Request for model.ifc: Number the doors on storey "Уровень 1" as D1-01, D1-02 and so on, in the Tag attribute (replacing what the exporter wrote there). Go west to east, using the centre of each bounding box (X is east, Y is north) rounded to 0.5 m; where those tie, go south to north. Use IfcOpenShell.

First a look at what the model holds.

```python
import ifcopenshell
import ifcopenshell.util.element
import ifcopenshell.util.placement

model = ifcopenshell.open("model.ifc")
print(model.schema)
storey = next(s for s in model.by_type("IfcBuildingStorey") if s.Name == "Уровень 1")
doors = [e for e in ifcopenshell.util.element.get_decomposition(storey) if e.is_a("IfcDoor")]
for e in sorted(doors, key=lambda e: e.id()):
    origin = ifcopenshell.util.placement.get_local_placement(e.ObjectPlacement)[:3, 3]
    print(e.id(), e.Tag, e.Name, origin.round(2) + 0.0, sep=" | ")
```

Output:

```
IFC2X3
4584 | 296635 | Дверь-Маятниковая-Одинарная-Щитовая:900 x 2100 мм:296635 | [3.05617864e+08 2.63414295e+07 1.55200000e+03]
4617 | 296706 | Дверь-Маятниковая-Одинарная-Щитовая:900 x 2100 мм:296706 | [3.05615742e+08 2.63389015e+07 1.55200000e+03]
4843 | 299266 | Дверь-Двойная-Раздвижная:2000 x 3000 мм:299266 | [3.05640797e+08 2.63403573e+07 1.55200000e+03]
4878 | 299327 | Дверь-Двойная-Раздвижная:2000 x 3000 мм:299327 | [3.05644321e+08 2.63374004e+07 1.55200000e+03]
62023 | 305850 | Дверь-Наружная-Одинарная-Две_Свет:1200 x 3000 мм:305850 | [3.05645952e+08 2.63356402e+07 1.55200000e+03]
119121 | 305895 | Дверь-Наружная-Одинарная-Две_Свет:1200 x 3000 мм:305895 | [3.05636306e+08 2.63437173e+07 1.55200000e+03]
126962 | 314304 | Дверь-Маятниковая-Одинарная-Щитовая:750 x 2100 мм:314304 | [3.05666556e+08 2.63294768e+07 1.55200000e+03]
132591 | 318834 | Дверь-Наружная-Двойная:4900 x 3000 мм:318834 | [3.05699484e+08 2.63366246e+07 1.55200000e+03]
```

```python
import ifcopenshell
import ifcopenshell.geom
import ifcopenshell.util.element
import ifcopenshell.util.shape

model = ifcopenshell.open("model.ifc")
settings = ifcopenshell.geom.settings()
settings.set("use-world-coords", True)


def centre(element):
    shape = ifcopenshell.geom.create_shape(settings, element)
    return ifcopenshell.util.shape.get_bbox_centroid(shape.geometry)


storey = next(s for s in model.by_type("IfcBuildingStorey") if s.Name == "Уровень 1")
doors = [e for e in ifcopenshell.util.element.get_decomposition(storey) if e.is_a("IfcDoor")]

# Insertion points can sit at a corner or the storey origin, so sort by the geometry (in metres).
centres = {e: centre(e) for e in doors}
doors.sort(key=lambda e: (round(centres[e][0] / 0.5), centres[e][1]))

for i, e in enumerate(doors, start=1):
    number = f"D1-{i:02d}"
    e.Tag = number
    print(e.id(), number)

model.write("model_v2.ifc")
```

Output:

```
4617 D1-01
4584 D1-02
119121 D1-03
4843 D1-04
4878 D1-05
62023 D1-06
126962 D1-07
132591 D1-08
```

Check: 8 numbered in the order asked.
